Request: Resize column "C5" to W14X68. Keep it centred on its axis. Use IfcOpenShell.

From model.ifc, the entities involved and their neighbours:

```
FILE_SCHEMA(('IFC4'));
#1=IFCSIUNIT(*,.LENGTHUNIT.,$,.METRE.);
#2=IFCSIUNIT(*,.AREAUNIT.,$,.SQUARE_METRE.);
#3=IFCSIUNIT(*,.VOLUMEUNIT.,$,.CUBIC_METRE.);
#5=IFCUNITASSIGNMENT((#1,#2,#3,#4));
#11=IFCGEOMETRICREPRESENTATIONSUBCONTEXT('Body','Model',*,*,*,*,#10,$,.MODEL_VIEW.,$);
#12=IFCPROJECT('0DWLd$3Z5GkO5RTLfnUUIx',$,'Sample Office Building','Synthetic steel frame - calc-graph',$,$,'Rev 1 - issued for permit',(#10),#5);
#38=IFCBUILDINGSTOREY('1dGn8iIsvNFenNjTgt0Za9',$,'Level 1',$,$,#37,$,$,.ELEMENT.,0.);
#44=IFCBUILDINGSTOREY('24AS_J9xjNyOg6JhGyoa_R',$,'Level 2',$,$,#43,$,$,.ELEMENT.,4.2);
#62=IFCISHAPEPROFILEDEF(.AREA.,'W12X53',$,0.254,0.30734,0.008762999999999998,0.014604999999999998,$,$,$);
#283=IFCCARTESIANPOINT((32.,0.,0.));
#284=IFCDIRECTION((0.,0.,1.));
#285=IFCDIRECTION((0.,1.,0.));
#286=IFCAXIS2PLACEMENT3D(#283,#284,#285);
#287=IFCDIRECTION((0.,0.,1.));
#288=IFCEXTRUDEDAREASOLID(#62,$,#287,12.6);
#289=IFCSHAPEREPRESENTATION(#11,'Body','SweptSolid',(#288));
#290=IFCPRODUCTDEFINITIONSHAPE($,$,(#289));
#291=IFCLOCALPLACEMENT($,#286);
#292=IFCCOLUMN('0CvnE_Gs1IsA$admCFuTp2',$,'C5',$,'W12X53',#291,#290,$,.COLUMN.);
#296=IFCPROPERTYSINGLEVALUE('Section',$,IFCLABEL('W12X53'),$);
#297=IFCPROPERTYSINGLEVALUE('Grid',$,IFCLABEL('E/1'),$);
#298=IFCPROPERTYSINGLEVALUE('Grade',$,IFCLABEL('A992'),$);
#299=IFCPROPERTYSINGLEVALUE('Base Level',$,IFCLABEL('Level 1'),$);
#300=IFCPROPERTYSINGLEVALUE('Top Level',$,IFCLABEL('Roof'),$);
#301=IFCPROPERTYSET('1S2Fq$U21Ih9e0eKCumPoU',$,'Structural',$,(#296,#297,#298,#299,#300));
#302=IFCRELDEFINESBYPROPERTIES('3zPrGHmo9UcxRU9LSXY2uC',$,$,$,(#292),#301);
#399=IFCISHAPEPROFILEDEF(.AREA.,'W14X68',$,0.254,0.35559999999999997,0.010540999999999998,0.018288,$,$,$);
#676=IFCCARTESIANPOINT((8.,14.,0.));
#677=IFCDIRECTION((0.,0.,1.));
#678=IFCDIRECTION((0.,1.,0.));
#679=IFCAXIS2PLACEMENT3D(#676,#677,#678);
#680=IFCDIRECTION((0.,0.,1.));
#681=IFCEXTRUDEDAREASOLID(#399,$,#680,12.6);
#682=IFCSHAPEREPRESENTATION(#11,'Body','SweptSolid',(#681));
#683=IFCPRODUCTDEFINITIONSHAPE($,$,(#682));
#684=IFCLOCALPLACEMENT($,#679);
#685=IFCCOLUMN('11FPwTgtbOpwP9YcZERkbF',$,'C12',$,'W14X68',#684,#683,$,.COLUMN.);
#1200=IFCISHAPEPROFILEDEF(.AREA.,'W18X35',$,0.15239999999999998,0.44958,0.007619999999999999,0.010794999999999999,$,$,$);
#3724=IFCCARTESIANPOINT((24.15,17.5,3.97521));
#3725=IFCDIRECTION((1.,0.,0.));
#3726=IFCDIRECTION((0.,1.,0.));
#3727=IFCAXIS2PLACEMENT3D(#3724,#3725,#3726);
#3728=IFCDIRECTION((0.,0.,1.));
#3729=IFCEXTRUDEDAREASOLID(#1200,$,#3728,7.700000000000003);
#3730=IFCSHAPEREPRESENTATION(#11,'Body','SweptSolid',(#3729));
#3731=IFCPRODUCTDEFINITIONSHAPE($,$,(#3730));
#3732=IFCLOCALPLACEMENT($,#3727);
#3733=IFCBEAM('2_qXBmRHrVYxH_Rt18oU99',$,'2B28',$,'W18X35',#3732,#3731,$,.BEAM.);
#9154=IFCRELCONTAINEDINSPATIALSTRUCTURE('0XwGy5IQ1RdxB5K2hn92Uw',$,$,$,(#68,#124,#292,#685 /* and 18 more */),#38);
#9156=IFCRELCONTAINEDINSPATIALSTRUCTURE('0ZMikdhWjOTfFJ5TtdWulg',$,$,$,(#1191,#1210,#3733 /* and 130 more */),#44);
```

```python
import ifcopenshell
import ifcopenshell.api.pset
import ifcopenshell.util.element
import ifcopenshell.util.representation

model = ifcopenshell.open("model.ifc")

member = model.by_id(292)
source = next(p for p in model.by_type("IfcIShapeProfileDef") if p.ProfileName == "W14X68")

body = ifcopenshell.util.representation.get_representation(member, "Model", "Body")
solid = body.Items[0]
old_profile = solid.SweptArea

# Copy the section's sizes but keep this member's own profile position.
profile = ifcopenshell.util.element.copy(model, source)
profile.Position = old_profile.Position
solid.SweptArea = profile
if not model.get_total_inverses(old_profile):
    ifcopenshell.util.element.remove_deep2(model, old_profile)
member.ObjectType = member.ObjectType.replace("W12X53", "W14X68")
pset = model.by_id(ifcopenshell.util.element.get_pset(member, "Structural", should_inherit=False)["id"])
ifcopenshell.api.pset.edit_pset(model, pset=pset, properties={"Section": "W14X68"})

print(solid.SweptArea)

model.write("model_updated.ifc")
```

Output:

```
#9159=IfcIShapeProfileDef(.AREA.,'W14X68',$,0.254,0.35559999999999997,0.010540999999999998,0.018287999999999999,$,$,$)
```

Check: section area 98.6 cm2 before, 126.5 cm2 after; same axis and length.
